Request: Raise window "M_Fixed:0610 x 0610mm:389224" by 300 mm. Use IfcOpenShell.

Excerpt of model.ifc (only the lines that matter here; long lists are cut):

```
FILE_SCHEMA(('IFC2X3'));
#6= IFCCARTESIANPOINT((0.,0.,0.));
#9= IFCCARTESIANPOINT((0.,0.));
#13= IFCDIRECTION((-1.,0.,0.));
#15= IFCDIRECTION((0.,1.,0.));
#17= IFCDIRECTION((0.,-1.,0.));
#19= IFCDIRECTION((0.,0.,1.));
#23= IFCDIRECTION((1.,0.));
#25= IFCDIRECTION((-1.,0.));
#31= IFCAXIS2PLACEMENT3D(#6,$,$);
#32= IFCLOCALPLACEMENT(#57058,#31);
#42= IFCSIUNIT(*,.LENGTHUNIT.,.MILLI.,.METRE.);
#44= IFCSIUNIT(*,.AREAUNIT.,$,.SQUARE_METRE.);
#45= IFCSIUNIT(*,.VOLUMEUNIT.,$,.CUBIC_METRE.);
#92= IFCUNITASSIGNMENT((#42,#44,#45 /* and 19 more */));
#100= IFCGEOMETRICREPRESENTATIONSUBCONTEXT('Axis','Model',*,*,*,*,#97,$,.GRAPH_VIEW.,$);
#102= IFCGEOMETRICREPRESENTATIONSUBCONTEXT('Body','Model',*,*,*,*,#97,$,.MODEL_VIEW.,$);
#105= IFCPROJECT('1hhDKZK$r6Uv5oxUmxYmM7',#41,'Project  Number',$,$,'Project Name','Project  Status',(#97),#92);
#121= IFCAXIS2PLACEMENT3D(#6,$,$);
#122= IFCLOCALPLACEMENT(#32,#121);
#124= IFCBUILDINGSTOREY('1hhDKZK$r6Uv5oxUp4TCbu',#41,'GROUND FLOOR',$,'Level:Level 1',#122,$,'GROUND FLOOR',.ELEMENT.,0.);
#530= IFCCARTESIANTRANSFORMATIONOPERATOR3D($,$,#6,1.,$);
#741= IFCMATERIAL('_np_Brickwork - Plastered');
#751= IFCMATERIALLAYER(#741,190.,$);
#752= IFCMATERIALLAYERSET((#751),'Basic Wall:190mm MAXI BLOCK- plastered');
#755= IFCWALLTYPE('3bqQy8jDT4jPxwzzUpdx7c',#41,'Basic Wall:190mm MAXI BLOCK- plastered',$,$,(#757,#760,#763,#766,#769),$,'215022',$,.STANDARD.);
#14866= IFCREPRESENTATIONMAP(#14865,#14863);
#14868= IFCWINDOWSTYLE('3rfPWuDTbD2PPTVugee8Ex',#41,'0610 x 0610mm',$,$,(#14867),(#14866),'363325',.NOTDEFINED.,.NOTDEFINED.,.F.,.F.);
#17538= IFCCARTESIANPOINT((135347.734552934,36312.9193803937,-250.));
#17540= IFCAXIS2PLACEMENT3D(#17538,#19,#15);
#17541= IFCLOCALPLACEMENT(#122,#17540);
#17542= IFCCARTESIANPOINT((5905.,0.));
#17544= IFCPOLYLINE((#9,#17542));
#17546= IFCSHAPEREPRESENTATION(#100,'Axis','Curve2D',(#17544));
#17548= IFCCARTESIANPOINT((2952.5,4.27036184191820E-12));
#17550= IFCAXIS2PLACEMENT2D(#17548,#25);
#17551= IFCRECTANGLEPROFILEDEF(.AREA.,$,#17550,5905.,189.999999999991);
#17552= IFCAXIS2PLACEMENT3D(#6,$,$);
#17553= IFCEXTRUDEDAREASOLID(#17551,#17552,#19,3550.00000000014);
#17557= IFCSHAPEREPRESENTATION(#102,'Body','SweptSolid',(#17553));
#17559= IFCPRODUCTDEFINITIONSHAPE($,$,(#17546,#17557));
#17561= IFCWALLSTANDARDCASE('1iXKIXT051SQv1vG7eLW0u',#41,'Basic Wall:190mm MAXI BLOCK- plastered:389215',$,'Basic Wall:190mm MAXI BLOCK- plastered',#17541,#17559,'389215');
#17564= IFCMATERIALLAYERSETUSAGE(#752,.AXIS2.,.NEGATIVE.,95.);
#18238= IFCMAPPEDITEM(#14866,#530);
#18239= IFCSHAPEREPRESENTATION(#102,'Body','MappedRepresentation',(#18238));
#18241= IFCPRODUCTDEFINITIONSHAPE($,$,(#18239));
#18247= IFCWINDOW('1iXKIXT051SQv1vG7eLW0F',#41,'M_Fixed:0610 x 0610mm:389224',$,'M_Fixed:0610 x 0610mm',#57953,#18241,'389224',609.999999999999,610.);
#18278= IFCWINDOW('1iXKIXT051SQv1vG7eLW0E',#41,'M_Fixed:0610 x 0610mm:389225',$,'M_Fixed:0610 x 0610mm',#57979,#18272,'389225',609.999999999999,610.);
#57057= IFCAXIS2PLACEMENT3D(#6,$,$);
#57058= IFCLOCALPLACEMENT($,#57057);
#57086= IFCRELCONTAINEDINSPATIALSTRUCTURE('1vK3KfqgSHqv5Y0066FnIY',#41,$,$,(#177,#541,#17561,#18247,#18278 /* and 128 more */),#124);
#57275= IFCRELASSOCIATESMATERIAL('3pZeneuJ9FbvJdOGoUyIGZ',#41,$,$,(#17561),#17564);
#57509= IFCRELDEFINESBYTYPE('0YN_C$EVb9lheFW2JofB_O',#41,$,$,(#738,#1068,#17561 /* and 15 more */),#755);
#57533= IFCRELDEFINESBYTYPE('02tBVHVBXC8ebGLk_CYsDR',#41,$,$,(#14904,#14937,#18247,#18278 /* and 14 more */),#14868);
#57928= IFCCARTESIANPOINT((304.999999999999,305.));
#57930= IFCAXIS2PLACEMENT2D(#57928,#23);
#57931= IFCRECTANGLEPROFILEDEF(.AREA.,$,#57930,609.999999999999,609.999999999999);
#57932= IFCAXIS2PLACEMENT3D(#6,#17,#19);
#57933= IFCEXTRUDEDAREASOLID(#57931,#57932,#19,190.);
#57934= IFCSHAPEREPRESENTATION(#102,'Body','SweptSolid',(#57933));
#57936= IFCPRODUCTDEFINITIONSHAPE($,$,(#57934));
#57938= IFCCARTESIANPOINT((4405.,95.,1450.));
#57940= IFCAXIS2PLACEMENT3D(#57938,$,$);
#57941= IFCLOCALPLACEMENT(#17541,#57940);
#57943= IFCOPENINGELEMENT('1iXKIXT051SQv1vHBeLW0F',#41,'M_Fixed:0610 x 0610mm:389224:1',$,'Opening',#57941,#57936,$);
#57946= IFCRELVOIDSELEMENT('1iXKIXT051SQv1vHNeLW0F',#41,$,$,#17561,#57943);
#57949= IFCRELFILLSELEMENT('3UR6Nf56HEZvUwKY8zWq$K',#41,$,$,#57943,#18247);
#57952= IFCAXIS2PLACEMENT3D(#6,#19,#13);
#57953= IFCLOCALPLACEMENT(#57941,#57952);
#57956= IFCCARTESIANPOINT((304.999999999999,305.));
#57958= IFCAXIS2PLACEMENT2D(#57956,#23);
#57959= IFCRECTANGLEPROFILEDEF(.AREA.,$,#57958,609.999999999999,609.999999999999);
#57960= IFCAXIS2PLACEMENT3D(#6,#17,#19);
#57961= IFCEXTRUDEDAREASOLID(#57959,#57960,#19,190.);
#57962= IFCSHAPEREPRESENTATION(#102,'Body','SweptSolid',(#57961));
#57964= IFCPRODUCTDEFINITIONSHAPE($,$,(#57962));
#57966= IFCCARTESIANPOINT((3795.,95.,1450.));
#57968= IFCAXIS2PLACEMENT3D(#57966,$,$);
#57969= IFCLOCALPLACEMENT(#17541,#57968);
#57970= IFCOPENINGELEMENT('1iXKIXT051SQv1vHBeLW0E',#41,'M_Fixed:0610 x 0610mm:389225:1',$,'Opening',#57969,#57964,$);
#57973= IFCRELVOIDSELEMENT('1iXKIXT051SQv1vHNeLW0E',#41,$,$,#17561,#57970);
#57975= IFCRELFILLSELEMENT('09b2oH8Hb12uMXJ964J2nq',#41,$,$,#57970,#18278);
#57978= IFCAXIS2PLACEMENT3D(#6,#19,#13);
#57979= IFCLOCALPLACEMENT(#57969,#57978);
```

```python
import numpy as np
import ifcopenshell
import ifcopenshell.api.geometry
import ifcopenshell.util.placement
import ifcopenshell.util.unit

model = ifcopenshell.open("model.ifc")
unit_scale = ifcopenshell.util.unit.calculate_unit_scale(model)

window = model.by_id(18247)
opening = window.FillsVoids[0].RelatingOpeningElement
dz = 0.3 / unit_scale

shift = np.array([0.0, 0.0, dz])
# The window is placed relative to its opening, so it follows when the opening moves.
matrix = ifcopenshell.util.placement.get_local_placement(opening.ObjectPlacement)
matrix[:3, 3] += shift
ifcopenshell.api.geometry.edit_object_placement(
    model, product=opening, matrix=matrix, is_si=False, should_transform_children=True
)

print(f"moved by {dz * unit_scale:+.3f} m")

model.write("model_rev.ifc")
```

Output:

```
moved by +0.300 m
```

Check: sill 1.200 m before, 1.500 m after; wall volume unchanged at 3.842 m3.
